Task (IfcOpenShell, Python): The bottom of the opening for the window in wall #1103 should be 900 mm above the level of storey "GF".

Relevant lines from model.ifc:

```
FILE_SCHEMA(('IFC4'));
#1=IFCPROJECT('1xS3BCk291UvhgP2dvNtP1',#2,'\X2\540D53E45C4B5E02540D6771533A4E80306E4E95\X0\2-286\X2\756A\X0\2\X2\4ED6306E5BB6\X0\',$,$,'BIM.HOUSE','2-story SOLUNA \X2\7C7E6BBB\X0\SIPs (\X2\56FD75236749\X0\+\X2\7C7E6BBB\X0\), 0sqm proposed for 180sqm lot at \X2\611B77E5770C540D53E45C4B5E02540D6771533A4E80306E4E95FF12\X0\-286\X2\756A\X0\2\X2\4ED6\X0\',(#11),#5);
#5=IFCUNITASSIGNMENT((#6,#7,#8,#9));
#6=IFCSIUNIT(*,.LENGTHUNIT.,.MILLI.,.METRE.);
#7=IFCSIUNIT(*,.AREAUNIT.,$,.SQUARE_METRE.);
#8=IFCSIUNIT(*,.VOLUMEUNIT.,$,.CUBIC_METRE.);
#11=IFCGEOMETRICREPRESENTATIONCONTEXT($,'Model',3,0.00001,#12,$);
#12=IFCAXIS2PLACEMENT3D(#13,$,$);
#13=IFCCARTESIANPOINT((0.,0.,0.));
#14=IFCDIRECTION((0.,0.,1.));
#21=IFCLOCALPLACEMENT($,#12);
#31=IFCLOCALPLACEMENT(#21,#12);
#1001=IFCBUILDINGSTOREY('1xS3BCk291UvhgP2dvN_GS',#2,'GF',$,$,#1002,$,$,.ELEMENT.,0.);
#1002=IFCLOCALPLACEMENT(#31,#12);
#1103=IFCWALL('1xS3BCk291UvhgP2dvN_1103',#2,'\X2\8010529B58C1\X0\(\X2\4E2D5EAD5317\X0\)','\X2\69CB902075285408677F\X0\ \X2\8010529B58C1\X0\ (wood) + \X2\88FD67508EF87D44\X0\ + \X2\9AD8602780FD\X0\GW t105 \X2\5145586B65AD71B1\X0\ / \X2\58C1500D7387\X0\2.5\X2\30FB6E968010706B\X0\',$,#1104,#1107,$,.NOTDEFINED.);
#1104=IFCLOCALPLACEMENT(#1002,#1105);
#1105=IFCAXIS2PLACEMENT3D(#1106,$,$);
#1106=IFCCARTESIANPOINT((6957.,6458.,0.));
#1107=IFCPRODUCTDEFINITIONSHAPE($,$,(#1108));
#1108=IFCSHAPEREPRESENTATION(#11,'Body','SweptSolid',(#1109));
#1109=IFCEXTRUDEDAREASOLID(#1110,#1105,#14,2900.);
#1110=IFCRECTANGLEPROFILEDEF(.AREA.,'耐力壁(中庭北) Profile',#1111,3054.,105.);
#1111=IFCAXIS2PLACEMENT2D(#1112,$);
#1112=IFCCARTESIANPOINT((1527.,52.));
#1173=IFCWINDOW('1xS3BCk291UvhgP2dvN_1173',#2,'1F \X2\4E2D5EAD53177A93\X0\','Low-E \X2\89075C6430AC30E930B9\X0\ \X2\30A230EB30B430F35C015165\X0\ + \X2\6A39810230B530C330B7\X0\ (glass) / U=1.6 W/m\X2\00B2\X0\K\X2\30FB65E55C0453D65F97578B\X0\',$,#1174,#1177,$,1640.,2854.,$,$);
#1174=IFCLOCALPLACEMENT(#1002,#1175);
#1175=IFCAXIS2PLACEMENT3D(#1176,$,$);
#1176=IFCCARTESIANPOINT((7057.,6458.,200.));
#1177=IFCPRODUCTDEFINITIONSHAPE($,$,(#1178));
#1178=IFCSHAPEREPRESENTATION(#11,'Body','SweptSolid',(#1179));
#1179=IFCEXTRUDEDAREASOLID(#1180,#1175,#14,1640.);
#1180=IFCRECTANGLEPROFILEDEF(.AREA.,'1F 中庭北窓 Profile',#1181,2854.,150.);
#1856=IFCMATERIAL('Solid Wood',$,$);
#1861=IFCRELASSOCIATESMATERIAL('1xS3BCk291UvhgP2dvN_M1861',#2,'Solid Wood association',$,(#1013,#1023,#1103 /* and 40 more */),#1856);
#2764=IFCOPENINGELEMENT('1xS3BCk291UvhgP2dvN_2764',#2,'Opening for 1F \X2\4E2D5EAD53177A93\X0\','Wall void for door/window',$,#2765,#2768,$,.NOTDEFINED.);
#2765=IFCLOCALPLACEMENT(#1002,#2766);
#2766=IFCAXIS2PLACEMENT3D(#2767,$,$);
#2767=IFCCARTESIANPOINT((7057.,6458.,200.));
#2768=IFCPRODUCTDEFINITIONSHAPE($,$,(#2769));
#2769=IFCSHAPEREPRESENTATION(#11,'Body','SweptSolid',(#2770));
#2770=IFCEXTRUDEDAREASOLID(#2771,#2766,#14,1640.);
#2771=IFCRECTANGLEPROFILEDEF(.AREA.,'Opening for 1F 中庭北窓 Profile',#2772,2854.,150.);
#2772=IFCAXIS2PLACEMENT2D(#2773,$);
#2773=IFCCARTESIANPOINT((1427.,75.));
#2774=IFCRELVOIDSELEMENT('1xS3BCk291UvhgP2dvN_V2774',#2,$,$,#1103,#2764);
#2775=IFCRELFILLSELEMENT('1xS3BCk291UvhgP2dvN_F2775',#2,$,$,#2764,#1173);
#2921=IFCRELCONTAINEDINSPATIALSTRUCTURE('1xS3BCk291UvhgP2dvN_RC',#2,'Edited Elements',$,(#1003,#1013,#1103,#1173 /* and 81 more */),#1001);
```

```python
import numpy as np
import ifcopenshell
import ifcopenshell.api.geometry
import ifcopenshell.geom
import ifcopenshell.util.element
import ifcopenshell.util.placement
import ifcopenshell.util.shape
import ifcopenshell.util.unit

model = ifcopenshell.open("model.ifc")
unit_scale = ifcopenshell.util.unit.calculate_unit_scale(model)

window = model.by_guid("1xS3BCk291UvhgP2dvN_1173")
opening = window.FillsVoids[0].RelatingOpeningElement
storey = ifcopenshell.util.element.get_container(window, ifc_class="IfcBuildingStorey")
level = ifcopenshell.util.placement.get_local_placement(storey.ObjectPlacement)[2, 3]

# The opening's origin need not be at the sill, so measure its lowest point.
shape = ifcopenshell.geom.create_shape(ifcopenshell.geom.settings(), opening)
bottom = ifcopenshell.util.shape.get_shape_bottom_elevation(shape, shape.geometry) / unit_scale
dz = level + 0.9 / unit_scale - bottom

shift = np.array([0.0, 0.0, dz])
# The window is not placed relative to its opening, so move both.
for product in (opening, window):
    matrix = ifcopenshell.util.placement.get_local_placement(product.ObjectPlacement)
    matrix[:3, 3] += shift
    ifcopenshell.api.geometry.edit_object_placement(model, product=product, matrix=matrix, is_si=False)

print(f"moved by {dz * unit_scale:+.3f} m")

model.write("model_edited.ifc")
```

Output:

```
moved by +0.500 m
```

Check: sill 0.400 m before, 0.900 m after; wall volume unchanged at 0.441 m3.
